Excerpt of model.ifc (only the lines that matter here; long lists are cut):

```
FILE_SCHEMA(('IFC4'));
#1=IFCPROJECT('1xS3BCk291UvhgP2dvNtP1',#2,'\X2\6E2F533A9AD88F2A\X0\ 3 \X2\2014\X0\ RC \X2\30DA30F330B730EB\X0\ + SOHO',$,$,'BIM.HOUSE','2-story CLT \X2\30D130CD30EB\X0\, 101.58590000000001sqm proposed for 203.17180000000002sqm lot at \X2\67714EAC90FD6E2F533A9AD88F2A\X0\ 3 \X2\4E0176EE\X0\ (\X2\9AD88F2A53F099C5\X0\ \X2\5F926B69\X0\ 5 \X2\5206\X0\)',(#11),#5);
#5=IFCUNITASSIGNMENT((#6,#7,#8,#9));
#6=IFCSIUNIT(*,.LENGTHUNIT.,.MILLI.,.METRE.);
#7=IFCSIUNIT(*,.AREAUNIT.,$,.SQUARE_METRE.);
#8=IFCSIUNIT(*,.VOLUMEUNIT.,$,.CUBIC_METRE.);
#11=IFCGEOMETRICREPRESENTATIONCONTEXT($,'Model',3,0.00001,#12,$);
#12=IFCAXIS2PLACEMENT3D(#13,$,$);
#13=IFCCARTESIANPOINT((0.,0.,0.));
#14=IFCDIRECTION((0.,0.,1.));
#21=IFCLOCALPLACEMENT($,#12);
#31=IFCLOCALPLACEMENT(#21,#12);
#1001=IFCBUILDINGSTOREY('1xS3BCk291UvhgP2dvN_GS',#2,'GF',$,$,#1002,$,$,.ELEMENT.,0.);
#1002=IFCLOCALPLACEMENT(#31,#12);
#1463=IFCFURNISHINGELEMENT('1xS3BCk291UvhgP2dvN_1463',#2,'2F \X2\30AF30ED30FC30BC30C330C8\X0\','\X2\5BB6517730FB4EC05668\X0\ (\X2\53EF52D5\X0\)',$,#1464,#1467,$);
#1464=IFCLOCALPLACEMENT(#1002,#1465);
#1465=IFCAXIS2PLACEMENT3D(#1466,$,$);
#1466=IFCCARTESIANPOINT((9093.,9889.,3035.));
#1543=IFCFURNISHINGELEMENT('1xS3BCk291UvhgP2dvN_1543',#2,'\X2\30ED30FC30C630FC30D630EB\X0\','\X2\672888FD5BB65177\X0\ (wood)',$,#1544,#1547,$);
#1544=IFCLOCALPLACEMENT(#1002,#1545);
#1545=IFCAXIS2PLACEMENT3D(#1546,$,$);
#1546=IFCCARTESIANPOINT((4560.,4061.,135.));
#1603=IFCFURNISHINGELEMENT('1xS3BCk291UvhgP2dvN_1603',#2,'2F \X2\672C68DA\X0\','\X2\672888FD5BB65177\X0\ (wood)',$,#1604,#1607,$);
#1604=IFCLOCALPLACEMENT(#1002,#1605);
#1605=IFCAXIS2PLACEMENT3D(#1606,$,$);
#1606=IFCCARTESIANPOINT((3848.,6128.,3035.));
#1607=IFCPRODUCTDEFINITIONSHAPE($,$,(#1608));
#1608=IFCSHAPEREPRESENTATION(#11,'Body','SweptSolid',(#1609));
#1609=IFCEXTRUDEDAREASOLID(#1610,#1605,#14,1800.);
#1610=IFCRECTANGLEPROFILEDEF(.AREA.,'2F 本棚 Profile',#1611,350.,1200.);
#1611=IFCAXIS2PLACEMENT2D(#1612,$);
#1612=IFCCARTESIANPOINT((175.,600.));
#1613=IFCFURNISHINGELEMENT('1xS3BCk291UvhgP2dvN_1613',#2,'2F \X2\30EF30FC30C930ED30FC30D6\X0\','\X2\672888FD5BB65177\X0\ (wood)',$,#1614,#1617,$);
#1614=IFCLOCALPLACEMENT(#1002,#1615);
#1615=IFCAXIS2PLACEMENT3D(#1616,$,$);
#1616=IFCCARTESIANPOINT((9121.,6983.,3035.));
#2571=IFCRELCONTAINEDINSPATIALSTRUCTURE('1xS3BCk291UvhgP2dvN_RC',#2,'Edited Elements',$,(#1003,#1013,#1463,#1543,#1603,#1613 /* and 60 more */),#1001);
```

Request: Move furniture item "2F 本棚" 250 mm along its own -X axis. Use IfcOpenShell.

```python
import ifcopenshell
import ifcopenshell.api.geometry
import ifcopenshell.util.placement
import ifcopenshell.util.unit

model = ifcopenshell.open("model.ifc")
unit_scale = ifcopenshell.util.unit.calculate_unit_scale(model)

item = model.by_id(1603)
matrix = ifcopenshell.util.placement.get_local_placement(item.ObjectPlacement)
matrix[:3, 3] -= matrix[:3, 0] * 0.25 / unit_scale
ifcopenshell.api.geometry.edit_object_placement(model, product=item, matrix=matrix, is_si=False)

print(ifcopenshell.util.placement.get_local_placement(item.ObjectPlacement).round(3) + 0.0)

model.write("model_rev.ifc")
```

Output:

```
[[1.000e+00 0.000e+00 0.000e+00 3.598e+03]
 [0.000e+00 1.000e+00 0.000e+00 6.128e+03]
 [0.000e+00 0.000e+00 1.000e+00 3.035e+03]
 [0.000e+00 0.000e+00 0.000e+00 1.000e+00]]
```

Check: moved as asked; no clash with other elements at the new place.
